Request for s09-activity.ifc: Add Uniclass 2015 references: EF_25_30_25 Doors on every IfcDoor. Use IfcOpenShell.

First a look at what the model holds.

```python
import ifcopenshell

model = ifcopenshell.open("s09-activity.ifc")
print(model.schema)
print("classifications:", [c.Name for c in model.by_type("IfcClassification")])
for ifc_class in ("IfcDoor", "IfcRoof", "IfcStair", "IfcWall", "IfcWindow"):
    print(ifc_class, len(model.by_type(ifc_class)))
```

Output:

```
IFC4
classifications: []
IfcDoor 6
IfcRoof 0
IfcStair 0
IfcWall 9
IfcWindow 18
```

```python
import ifcopenshell
import ifcopenshell.api.classification

model = ifcopenshell.open("s09-activity.ifc")

system = ifcopenshell.api.classification.add_classification(model, classification="Uniclass 2015")

codes = {
    "IfcDoor": ("EF_25_30_25", "Doors"),
}
for ifc_class, (code, name) in codes.items():
    products = model.by_type(ifc_class)
    ifcopenshell.api.classification.add_reference(
        model, products=products, classification=system, identification=code, name=name
    )
    print(code, len(products))

model.write("s09-activity_updated.ifc")
```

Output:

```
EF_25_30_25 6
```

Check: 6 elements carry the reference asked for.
